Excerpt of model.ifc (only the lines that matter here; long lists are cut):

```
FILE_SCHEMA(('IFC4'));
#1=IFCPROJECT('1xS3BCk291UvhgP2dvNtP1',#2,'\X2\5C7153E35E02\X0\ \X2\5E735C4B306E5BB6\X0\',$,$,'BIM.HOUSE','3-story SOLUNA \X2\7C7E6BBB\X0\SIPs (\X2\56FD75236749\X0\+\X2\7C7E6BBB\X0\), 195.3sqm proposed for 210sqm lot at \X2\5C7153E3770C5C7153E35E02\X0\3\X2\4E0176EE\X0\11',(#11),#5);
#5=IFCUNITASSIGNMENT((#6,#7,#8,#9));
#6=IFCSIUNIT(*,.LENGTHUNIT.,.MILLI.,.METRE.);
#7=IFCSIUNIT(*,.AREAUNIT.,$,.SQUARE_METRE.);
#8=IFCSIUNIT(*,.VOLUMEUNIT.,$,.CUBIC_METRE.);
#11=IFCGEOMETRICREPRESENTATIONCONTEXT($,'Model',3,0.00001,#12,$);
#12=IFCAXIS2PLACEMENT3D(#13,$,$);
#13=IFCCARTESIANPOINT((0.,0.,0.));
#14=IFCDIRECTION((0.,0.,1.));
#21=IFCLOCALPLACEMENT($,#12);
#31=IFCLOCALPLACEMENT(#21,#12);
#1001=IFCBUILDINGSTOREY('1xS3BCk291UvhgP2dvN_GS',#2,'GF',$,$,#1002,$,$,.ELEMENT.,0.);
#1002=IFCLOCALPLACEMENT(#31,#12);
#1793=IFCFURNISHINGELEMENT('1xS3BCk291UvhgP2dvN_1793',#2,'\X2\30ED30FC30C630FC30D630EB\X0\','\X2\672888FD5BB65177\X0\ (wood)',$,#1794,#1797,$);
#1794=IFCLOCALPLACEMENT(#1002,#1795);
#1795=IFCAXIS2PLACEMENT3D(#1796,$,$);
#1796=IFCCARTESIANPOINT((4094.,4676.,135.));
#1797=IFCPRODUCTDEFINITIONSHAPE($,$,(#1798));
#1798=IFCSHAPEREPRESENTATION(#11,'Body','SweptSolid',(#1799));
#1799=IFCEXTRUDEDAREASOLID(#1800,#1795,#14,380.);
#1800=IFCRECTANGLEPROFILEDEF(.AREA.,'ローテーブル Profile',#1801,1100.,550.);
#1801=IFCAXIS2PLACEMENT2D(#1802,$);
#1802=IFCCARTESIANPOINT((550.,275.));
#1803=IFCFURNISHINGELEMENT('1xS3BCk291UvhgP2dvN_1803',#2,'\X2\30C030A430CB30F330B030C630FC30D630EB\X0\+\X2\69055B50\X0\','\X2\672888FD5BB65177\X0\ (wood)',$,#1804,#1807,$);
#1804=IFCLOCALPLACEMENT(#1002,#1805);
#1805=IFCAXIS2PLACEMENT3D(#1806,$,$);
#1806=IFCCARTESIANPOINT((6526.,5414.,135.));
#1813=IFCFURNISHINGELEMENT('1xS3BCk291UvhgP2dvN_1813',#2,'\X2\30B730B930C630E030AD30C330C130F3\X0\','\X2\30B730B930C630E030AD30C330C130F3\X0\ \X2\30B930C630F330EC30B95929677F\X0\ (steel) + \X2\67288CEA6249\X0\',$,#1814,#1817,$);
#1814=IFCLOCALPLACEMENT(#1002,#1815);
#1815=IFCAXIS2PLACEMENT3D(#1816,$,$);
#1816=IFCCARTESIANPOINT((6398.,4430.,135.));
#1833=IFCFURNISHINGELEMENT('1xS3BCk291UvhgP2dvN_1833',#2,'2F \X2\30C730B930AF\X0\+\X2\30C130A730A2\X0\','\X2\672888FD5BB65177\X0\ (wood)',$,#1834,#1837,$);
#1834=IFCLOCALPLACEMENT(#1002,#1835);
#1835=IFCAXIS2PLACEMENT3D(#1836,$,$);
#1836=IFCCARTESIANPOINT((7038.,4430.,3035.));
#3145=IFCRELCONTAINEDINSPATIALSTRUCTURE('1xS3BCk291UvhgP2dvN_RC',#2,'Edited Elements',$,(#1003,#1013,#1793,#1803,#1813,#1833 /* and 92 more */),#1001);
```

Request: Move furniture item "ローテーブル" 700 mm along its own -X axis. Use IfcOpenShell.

```python
import ifcopenshell
import ifcopenshell.api.geometry
import ifcopenshell.util.placement

model = ifcopenshell.open("model.ifc")

item = model.by_guid("1xS3BCk291UvhgP2dvN_1793")
matrix = ifcopenshell.util.placement.get_local_placement(item.ObjectPlacement)
matrix[:3, 3] -= matrix[:3, 0] * 700.0
ifcopenshell.api.geometry.edit_object_placement(model, product=item, matrix=matrix, is_si=False)

print(ifcopenshell.util.placement.get_local_placement(item.ObjectPlacement).round(3) + 0.0)

model.write("model_v2.ifc")
```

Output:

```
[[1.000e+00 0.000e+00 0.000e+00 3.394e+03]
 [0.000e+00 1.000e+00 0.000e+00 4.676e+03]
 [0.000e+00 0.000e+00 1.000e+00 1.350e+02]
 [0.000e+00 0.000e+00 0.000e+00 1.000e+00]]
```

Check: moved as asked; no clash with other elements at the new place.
